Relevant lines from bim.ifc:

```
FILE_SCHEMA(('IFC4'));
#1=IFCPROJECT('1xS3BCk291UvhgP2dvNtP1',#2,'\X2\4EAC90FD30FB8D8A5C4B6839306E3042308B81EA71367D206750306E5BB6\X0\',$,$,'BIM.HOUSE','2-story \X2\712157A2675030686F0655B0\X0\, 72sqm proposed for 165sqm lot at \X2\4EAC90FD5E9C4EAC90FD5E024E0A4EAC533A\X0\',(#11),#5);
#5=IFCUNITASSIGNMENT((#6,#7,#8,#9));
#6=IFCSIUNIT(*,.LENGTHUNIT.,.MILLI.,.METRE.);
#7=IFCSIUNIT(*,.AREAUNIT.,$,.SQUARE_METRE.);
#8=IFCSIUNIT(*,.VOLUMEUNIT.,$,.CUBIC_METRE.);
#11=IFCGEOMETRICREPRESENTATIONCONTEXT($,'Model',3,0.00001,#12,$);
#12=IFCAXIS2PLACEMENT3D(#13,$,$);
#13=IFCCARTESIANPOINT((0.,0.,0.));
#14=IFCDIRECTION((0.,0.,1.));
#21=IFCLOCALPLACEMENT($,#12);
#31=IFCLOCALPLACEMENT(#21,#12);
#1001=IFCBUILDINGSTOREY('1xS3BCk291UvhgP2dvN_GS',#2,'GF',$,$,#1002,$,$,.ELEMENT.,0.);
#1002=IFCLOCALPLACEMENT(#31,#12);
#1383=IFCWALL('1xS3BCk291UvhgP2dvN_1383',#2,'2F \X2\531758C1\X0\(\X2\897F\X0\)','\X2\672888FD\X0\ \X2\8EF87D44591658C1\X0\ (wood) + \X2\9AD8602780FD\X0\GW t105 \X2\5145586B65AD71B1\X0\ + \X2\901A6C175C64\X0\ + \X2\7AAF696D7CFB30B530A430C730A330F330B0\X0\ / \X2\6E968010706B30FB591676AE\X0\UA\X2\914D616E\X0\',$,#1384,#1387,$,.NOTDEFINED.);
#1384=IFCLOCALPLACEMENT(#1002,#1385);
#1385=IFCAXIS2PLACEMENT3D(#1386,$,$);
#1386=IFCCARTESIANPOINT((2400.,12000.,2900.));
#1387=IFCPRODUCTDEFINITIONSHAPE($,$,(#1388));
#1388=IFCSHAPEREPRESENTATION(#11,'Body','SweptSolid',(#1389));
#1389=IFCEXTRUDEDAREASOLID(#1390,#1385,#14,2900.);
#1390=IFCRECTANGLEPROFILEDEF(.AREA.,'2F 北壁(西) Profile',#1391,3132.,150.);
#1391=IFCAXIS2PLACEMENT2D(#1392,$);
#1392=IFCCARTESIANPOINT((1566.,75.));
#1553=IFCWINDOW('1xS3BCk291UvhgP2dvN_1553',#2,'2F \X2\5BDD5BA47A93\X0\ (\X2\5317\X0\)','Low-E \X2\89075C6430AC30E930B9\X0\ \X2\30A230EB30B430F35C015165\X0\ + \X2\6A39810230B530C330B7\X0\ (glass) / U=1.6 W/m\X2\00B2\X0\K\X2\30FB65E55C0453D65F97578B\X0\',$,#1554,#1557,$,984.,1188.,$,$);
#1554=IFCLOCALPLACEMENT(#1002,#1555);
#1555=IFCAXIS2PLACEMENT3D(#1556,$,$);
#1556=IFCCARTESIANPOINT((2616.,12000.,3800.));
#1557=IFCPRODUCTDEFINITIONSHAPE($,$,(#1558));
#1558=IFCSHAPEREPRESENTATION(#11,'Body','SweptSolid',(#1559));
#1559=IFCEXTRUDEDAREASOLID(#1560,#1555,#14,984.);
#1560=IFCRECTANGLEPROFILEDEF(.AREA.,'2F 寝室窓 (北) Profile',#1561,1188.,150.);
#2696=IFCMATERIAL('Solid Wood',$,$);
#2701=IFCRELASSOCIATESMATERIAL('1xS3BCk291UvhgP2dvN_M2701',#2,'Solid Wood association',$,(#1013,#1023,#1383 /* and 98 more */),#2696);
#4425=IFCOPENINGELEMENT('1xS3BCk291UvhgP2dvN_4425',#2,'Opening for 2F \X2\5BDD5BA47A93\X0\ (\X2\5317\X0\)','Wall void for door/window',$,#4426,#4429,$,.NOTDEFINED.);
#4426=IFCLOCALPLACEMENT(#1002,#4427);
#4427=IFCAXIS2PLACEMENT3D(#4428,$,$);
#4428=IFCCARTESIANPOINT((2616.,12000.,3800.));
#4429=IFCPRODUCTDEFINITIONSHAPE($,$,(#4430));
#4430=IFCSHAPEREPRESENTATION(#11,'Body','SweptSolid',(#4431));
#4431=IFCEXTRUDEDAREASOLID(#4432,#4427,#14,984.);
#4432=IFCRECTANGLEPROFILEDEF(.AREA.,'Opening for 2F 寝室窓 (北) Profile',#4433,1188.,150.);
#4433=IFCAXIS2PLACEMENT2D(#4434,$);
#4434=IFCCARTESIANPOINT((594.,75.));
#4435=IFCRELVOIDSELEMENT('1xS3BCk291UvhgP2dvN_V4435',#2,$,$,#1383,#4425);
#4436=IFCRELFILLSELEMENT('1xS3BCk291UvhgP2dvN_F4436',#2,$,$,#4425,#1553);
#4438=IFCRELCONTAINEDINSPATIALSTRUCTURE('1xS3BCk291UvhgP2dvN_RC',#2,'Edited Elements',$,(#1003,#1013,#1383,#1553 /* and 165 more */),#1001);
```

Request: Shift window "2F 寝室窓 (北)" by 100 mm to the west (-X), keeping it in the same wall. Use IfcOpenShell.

```python
import ifcopenshell
import ifcopenshell.api.geometry
import ifcopenshell.util.placement
import ifcopenshell.util.unit

model = ifcopenshell.open("bim.ifc")
unit_scale = ifcopenshell.util.unit.calculate_unit_scale(model)

window = model.by_guid("1xS3BCk291UvhgP2dvN_1553")
opening = window.FillsVoids[0].RelatingOpeningElement
wall = opening.VoidsElements[0].RelatingBuildingElement

wall_matrix = ifcopenshell.util.placement.get_local_placement(wall.ObjectPlacement)
shift = wall_matrix[:3, 0] * -0.1 / unit_scale
before = ifcopenshell.util.placement.get_local_placement(window.ObjectPlacement)[:3, 3].copy()

# The window is not placed relative to its opening, so move both.
for product in (opening, window):
    matrix = ifcopenshell.util.placement.get_local_placement(product.ObjectPlacement)
    matrix[:3, 3] += shift
    ifcopenshell.api.geometry.edit_object_placement(model, product=product, matrix=matrix, is_si=False)

after = ifcopenshell.util.placement.get_local_placement(window.ObjectPlacement)[:3, 3]
print("window moved by", (after - before).round(3) + 0.0)

model.write("bim_rev.ifc")
```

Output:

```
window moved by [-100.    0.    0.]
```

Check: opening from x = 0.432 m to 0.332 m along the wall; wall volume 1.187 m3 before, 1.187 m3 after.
